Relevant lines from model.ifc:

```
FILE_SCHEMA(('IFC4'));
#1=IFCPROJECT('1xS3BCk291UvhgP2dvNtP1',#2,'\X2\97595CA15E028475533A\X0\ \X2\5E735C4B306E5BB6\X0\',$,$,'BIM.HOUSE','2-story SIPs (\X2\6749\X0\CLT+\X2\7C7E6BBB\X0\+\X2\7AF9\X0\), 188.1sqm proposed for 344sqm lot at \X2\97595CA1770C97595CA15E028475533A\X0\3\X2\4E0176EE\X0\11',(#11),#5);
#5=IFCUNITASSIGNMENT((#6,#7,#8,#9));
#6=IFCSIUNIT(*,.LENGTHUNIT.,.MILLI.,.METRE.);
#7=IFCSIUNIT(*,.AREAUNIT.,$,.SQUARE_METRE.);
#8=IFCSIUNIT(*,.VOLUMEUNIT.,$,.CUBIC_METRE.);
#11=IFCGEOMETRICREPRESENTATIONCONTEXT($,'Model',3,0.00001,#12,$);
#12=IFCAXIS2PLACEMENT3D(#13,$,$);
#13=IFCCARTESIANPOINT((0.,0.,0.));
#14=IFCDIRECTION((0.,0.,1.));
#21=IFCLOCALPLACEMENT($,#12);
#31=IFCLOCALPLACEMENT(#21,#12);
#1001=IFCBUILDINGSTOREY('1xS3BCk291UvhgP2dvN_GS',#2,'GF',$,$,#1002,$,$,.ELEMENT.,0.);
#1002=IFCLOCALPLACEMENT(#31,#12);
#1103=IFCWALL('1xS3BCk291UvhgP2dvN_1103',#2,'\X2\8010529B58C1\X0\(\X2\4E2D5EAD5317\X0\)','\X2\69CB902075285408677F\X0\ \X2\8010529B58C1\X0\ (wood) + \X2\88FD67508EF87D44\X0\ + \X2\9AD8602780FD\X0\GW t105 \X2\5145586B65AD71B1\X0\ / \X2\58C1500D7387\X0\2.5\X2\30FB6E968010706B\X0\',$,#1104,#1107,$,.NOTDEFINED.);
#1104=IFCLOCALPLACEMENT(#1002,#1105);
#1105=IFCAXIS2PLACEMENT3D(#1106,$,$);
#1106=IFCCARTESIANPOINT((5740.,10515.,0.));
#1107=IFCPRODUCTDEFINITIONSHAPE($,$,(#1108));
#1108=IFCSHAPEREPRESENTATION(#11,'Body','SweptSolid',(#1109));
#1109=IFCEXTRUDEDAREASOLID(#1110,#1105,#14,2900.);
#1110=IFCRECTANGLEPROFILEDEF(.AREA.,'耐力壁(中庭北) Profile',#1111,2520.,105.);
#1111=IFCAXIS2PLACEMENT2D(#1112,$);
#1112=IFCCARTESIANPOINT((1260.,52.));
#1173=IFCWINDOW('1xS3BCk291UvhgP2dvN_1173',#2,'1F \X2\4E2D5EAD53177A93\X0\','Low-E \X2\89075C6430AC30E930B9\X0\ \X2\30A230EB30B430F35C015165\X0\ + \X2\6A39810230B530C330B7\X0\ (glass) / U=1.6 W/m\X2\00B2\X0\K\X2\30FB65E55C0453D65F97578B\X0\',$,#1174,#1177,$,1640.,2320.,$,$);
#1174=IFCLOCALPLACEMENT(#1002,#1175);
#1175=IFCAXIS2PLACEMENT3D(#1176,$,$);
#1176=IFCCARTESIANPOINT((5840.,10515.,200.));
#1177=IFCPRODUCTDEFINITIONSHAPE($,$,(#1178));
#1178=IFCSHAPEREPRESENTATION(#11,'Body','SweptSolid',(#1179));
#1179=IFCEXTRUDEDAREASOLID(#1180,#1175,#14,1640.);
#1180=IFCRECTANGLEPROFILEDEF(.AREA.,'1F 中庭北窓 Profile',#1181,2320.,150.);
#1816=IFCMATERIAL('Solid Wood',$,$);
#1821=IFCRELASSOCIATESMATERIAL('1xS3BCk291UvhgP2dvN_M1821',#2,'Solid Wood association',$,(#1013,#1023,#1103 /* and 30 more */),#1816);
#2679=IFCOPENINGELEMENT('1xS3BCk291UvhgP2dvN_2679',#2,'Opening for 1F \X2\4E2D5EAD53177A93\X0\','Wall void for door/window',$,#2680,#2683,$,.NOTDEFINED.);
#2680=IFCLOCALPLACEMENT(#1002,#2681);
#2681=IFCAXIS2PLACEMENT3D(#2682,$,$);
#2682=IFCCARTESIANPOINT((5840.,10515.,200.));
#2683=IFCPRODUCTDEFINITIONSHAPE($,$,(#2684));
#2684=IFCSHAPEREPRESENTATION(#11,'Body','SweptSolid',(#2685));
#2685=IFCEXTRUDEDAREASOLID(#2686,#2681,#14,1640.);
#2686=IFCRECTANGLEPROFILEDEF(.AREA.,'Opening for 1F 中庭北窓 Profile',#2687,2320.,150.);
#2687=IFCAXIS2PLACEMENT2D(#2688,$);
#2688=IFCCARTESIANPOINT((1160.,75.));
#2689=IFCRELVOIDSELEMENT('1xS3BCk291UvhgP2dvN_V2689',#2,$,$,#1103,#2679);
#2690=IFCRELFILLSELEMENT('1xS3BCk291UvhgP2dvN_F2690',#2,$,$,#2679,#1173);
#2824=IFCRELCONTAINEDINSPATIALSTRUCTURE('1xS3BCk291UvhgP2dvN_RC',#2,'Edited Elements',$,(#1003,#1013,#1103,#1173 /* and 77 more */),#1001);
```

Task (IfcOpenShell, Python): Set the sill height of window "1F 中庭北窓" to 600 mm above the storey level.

```python
import numpy as np
import ifcopenshell
import ifcopenshell.api.geometry
import ifcopenshell.geom
import ifcopenshell.util.element
import ifcopenshell.util.placement
import ifcopenshell.util.shape
import ifcopenshell.util.unit

model = ifcopenshell.open("model.ifc")
unit_scale = ifcopenshell.util.unit.calculate_unit_scale(model)

window = model.by_guid("1xS3BCk291UvhgP2dvN_1173")
opening = window.FillsVoids[0].RelatingOpeningElement
storey = ifcopenshell.util.element.get_container(window, ifc_class="IfcBuildingStorey")
level = ifcopenshell.util.placement.get_local_placement(storey.ObjectPlacement)[2, 3]

# The opening's origin need not be at the sill, so measure its lowest point.
shape = ifcopenshell.geom.create_shape(ifcopenshell.geom.settings(), opening)
bottom = ifcopenshell.util.shape.get_shape_bottom_elevation(shape, shape.geometry) / unit_scale
dz = level + 0.6 / unit_scale - bottom

shift = np.array([0.0, 0.0, dz])
# The window is not placed relative to its opening, so move both.
for product in (opening, window):
    matrix = ifcopenshell.util.placement.get_local_placement(product.ObjectPlacement)
    matrix[:3, 3] += shift
    ifcopenshell.api.geometry.edit_object_placement(model, product=product, matrix=matrix, is_si=False)

print(f"moved by {dz * unit_scale:+.3f} m")

model.write("model_v2.ifc")
```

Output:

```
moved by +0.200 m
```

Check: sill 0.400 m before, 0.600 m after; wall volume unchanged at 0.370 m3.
